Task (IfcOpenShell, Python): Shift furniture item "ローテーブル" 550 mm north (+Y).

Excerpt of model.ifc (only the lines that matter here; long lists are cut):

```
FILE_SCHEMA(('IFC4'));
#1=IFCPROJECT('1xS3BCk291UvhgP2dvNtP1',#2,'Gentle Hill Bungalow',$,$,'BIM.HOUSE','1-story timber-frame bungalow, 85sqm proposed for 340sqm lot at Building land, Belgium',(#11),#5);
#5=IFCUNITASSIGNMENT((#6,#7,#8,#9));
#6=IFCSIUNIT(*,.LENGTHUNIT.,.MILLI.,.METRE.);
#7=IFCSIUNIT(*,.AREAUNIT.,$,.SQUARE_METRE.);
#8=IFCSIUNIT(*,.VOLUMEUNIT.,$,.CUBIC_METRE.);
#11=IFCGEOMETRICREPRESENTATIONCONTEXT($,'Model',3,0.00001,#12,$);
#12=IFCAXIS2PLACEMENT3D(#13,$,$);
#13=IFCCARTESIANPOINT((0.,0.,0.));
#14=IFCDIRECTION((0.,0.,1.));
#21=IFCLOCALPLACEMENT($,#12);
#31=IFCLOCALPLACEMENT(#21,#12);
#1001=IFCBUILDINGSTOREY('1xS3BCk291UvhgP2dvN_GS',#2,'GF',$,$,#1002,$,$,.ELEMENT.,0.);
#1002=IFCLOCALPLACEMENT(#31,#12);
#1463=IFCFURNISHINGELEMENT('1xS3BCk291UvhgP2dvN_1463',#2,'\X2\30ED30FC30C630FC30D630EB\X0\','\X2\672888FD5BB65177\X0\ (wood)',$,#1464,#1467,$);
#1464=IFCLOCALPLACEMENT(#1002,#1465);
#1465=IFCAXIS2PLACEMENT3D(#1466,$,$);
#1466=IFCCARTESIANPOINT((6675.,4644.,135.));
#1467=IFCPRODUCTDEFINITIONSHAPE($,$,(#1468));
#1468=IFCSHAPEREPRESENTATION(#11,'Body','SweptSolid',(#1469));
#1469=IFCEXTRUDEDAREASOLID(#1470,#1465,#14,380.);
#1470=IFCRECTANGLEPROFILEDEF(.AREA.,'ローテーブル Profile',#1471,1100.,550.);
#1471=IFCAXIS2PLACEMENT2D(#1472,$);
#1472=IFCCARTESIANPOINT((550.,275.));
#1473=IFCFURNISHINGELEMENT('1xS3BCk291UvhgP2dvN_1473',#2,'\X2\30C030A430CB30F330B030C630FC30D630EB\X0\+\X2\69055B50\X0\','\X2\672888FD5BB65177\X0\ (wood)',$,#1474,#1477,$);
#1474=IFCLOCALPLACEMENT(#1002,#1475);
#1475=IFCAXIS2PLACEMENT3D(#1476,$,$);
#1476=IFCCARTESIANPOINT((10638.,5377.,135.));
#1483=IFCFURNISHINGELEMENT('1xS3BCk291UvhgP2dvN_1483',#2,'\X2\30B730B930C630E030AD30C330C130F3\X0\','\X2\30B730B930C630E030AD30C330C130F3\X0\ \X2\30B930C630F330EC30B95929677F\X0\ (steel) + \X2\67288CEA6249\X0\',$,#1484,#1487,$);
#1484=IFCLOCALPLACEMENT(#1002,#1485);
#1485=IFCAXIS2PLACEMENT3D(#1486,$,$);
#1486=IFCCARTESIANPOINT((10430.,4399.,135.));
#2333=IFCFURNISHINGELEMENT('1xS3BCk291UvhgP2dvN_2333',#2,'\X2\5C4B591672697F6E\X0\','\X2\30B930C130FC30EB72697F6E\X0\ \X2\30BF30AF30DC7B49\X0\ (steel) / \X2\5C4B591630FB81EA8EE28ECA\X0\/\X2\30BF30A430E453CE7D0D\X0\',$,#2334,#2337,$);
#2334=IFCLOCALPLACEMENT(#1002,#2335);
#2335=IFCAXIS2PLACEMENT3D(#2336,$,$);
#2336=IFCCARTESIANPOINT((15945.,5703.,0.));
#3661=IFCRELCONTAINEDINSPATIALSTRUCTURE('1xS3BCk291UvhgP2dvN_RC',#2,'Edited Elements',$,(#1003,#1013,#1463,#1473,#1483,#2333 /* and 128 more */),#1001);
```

```python
import ifcopenshell
import ifcopenshell.api.geometry
import ifcopenshell.util.placement
import ifcopenshell.util.unit

model = ifcopenshell.open("model.ifc")
unit_scale = ifcopenshell.util.unit.calculate_unit_scale(model)

item = model.by_id(1463)
matrix = ifcopenshell.util.placement.get_local_placement(item.ObjectPlacement)
matrix[1, 3] += 0.55 / unit_scale
ifcopenshell.api.geometry.edit_object_placement(model, product=item, matrix=matrix, is_si=False)

print(ifcopenshell.util.placement.get_local_placement(item.ObjectPlacement).round(3) + 0.0)

model.write("model_updated.ifc")
```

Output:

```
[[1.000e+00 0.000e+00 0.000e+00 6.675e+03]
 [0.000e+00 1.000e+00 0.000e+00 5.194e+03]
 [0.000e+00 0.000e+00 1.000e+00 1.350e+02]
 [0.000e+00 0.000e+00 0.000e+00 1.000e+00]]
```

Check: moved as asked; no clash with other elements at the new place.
